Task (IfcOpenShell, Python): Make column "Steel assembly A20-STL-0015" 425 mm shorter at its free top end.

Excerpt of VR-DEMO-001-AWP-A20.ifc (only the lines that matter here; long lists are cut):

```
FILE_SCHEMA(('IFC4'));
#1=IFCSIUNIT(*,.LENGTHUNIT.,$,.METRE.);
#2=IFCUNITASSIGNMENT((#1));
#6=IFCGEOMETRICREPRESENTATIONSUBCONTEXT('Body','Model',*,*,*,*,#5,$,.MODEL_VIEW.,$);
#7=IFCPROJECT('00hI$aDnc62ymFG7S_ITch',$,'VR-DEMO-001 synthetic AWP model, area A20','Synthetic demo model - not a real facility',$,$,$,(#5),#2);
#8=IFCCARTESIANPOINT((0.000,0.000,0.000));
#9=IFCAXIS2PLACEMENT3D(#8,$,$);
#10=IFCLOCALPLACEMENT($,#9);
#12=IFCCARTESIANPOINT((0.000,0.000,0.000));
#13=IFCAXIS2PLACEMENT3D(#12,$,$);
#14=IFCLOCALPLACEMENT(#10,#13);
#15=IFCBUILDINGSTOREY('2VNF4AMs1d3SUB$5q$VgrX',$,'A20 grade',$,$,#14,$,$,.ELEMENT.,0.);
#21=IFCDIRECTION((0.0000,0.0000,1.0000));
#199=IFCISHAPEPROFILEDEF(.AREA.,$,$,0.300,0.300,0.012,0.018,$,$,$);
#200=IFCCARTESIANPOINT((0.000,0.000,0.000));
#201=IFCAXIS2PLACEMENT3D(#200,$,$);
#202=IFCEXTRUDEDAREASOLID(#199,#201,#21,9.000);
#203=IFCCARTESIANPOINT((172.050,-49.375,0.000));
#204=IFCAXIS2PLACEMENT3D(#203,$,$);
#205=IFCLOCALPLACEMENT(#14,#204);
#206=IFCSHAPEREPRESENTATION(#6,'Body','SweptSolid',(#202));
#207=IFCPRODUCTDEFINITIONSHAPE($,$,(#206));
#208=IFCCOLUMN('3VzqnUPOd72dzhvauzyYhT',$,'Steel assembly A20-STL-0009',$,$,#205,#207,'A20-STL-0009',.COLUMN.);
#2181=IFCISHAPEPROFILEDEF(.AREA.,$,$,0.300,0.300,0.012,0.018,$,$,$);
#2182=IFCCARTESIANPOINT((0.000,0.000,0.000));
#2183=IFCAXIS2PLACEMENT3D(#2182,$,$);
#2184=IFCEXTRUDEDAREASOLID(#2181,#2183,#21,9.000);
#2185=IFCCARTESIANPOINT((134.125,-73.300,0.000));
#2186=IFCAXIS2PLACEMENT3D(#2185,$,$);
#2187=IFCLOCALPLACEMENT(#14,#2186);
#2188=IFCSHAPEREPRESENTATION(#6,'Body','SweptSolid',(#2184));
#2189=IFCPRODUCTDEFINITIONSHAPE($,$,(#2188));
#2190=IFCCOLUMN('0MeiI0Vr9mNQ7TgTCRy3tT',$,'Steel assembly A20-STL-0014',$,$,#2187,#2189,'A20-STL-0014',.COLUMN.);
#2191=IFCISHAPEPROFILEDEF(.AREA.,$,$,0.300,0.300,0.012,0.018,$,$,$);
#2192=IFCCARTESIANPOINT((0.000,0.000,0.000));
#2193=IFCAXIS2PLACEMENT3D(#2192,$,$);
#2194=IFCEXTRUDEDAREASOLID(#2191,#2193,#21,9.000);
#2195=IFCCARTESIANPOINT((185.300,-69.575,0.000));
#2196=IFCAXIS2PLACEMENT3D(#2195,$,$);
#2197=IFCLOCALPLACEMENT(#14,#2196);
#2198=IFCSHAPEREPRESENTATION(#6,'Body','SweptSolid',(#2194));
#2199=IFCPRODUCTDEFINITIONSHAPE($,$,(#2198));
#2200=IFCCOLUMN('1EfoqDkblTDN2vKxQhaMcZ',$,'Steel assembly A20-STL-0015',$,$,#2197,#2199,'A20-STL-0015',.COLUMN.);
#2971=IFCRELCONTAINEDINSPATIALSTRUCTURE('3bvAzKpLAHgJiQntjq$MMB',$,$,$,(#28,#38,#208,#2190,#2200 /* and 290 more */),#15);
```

```python
import ifcopenshell
import ifcopenshell.util.representation

model = ifcopenshell.open("VR-DEMO-001-AWP-A20.ifc")

member = model.by_guid("1EfoqDkblTDN2vKxQhaMcZ")
change = -0.425

# The extrusion runs towards the end named, so only its depth changes.
body = ifcopenshell.util.representation.get_representation(member, "Model", "Body")
solid = body.Items[0]
old_length = solid.Depth
solid.Depth += change

print(f"length {old_length:g} -> {solid.Depth:g}")

model.write("VR-DEMO-001-AWP-A20-out.ifc")
```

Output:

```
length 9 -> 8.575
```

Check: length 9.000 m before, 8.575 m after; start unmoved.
